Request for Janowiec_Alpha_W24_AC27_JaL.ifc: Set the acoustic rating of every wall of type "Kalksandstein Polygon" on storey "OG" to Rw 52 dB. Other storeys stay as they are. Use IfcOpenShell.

First a look at what the model holds.

```python
import ifcopenshell
import ifcopenshell.util.element

model = ifcopenshell.open("Janowiec_Alpha_W24_AC27_JaL.ifc")
print(model.schema)
storey = next(s for s in model.by_type("IfcBuildingStorey") if s.Name == "OG")
walls = [e for e in ifcopenshell.util.element.get_decomposition(storey) if e.is_a("IfcWall")]
seen = {}
for e in walls:
    element_type = ifcopenshell.util.element.get_type(e)
    key = (element_type.Name if element_type != e and element_type else None, ifcopenshell.util.element.get_pset(e, "Pset_WallCommon", "AcousticRating"))
    seen[key] = seen.get(key, 0) + 1
for (name, value), count in sorted(seen.items(), key=str):
    print(count, "x", name, "|", value)
```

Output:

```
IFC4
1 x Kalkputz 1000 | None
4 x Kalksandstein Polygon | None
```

```python
import ifcopenshell
import ifcopenshell.api.pset
import ifcopenshell.util.element

model = ifcopenshell.open("Janowiec_Alpha_W24_AC27_JaL.ifc")

storey = next(s for s in model.by_type("IfcBuildingStorey") if s.Name == "OG")
walls = [e for e in ifcopenshell.util.element.get_decomposition(storey) if e.is_a("IfcWall")]

count = 0
for e in walls:
    element_type = ifcopenshell.util.element.get_type(e)
    if element_type in (None, e) or element_type.Name != "Kalksandstein Polygon":
        continue
    # add_pset returns the element's existing set when there is one.
    pset = ifcopenshell.api.pset.add_pset(model, product=e, name="Pset_WallCommon")
    ifcopenshell.api.pset.edit_pset(model, pset=pset, properties={"AcousticRating": "Rw 52 dB"})
    count += 1

print(count, "walls updated")

model.write("Janowiec_Alpha_W24_AC27_JaL_updated.ifc")
```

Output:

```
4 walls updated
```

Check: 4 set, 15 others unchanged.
